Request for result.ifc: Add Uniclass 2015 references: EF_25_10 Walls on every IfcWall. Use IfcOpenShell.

First a look at what the model holds.

```python
import ifcopenshell

model = ifcopenshell.open("result.ifc")
print(model.schema)
print("classifications:", [c.Name for c in model.by_type("IfcClassification")])
for ifc_class in ("IfcDoor", "IfcRoof", "IfcStair", "IfcWall", "IfcWindow"):
    print(ifc_class, len(model.by_type(ifc_class)))
```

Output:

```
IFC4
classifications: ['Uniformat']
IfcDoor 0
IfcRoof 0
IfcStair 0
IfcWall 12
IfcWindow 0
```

```python
import ifcopenshell
import ifcopenshell.api.classification

model = ifcopenshell.open("result.ifc")

system = ifcopenshell.api.classification.add_classification(model, classification="Uniclass 2015")

codes = {
    "IfcWall": ("EF_25_10", "Walls"),
}
for ifc_class, (code, name) in codes.items():
    products = model.by_type(ifc_class)
    ifcopenshell.api.classification.add_reference(
        model, products=products, classification=system, identification=code, name=name
    )
    print(code, len(products))

model.write("result-out.ifc")
```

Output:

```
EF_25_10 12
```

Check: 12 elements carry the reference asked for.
